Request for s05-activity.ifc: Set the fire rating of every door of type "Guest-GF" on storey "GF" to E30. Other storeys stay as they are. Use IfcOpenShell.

First a look at what the model holds.

```python
import ifcopenshell
import ifcopenshell.util.element

model = ifcopenshell.open("s05-activity.ifc")
print(model.schema)
storey = next(s for s in model.by_type("IfcBuildingStorey") if s.Name == "GF")
doors = [e for e in ifcopenshell.util.element.get_decomposition(storey) if e.is_a("IfcDoor")]
seen = {}
for e in doors:
    element_type = ifcopenshell.util.element.get_type(e)
    key = (element_type.Name if element_type != e and element_type else None, ifcopenshell.util.element.get_pset(e, "Pset_DoorCommon", "FireRating"))
    seen[key] = seen.get(key, 0) + 1
for (name, value), count in sorted(seen.items(), key=str):
    print(count, "x", name, "|", value)
```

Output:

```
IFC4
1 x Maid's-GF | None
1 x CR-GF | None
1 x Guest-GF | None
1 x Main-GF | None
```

```python
import ifcopenshell
import ifcopenshell.api.pset
import ifcopenshell.util.element

model = ifcopenshell.open("s05-activity.ifc")

storey = next(s for s in model.by_type("IfcBuildingStorey") if s.Name == "GF")
doors = [e for e in ifcopenshell.util.element.get_decomposition(storey) if e.is_a("IfcDoor")]

count = 0
for e in doors:
    element_type = ifcopenshell.util.element.get_type(e)
    if element_type in (None, e) or element_type.Name != "Guest-GF":
        continue
    # add_pset returns the element's existing set when there is one.
    pset = ifcopenshell.api.pset.add_pset(model, product=e, name="Pset_DoorCommon")
    ifcopenshell.api.pset.edit_pset(model, pset=pset, properties={"FireRating": "E30"})
    count += 1

print(count, "doors updated")

model.write("s05-activity-out.ifc")
```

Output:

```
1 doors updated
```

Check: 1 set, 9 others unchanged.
